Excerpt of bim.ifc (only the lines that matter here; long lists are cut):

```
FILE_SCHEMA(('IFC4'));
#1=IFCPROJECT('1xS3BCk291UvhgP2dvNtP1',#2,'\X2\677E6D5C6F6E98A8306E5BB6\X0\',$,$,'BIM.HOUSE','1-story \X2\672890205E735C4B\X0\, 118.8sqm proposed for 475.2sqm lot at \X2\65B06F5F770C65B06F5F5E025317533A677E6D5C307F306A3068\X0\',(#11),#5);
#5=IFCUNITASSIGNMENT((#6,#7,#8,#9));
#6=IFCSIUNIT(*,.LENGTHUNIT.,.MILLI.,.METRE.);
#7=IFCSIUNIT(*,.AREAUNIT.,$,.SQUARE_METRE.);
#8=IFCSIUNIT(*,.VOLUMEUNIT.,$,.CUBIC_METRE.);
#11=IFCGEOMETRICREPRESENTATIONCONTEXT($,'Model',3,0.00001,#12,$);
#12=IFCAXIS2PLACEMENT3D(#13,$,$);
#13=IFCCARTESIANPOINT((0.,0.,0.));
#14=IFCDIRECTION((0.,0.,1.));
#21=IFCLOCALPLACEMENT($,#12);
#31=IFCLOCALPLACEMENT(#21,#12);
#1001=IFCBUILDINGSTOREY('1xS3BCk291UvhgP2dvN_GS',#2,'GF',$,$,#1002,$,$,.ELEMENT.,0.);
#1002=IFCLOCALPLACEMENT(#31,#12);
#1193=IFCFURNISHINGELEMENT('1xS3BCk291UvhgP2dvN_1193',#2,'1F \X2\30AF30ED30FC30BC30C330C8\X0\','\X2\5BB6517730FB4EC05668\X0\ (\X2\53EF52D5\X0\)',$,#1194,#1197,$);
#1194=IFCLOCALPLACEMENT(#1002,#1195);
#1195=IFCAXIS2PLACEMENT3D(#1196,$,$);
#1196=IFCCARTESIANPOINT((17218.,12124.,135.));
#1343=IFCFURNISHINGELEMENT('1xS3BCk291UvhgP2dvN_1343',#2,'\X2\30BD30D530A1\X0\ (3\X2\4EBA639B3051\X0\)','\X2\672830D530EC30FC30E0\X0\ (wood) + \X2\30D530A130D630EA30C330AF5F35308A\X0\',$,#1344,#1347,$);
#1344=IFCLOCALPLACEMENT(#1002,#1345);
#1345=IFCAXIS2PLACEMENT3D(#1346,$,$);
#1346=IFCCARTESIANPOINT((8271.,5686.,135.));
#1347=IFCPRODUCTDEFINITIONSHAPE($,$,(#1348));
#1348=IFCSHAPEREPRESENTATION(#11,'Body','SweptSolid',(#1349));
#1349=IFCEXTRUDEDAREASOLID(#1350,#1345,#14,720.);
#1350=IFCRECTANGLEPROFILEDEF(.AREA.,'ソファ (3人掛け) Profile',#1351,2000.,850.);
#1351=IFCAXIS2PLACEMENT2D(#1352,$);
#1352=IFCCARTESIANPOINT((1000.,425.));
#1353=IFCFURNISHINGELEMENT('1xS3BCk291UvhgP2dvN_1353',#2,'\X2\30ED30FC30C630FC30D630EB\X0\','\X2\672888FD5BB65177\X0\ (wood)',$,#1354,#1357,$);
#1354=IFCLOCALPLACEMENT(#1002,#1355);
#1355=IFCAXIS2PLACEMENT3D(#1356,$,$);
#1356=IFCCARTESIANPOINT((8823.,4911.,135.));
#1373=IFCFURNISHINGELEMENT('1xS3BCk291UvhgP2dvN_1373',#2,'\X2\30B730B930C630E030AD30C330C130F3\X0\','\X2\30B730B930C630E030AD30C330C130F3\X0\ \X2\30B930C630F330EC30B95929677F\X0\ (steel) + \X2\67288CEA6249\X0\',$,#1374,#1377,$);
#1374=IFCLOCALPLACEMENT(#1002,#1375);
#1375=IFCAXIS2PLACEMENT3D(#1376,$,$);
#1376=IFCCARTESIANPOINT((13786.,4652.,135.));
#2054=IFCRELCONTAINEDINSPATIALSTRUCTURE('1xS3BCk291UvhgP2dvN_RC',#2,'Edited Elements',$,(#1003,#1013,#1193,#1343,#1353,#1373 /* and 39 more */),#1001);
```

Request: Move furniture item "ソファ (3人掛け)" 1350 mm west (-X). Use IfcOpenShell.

```python
import ifcopenshell
import ifcopenshell.api.geometry
import ifcopenshell.util.placement

model = ifcopenshell.open("bim.ifc")

item = model.by_guid("1xS3BCk291UvhgP2dvN_1343")
matrix = ifcopenshell.util.placement.get_local_placement(item.ObjectPlacement)
matrix[0, 3] -= 1350.0
ifcopenshell.api.geometry.edit_object_placement(model, product=item, matrix=matrix, is_si=False)

print(ifcopenshell.util.placement.get_local_placement(item.ObjectPlacement).round(3) + 0.0)

model.write("bim_updated.ifc")
```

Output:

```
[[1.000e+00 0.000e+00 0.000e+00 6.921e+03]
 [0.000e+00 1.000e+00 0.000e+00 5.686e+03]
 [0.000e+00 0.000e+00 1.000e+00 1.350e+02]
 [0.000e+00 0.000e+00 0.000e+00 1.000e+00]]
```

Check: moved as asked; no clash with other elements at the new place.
